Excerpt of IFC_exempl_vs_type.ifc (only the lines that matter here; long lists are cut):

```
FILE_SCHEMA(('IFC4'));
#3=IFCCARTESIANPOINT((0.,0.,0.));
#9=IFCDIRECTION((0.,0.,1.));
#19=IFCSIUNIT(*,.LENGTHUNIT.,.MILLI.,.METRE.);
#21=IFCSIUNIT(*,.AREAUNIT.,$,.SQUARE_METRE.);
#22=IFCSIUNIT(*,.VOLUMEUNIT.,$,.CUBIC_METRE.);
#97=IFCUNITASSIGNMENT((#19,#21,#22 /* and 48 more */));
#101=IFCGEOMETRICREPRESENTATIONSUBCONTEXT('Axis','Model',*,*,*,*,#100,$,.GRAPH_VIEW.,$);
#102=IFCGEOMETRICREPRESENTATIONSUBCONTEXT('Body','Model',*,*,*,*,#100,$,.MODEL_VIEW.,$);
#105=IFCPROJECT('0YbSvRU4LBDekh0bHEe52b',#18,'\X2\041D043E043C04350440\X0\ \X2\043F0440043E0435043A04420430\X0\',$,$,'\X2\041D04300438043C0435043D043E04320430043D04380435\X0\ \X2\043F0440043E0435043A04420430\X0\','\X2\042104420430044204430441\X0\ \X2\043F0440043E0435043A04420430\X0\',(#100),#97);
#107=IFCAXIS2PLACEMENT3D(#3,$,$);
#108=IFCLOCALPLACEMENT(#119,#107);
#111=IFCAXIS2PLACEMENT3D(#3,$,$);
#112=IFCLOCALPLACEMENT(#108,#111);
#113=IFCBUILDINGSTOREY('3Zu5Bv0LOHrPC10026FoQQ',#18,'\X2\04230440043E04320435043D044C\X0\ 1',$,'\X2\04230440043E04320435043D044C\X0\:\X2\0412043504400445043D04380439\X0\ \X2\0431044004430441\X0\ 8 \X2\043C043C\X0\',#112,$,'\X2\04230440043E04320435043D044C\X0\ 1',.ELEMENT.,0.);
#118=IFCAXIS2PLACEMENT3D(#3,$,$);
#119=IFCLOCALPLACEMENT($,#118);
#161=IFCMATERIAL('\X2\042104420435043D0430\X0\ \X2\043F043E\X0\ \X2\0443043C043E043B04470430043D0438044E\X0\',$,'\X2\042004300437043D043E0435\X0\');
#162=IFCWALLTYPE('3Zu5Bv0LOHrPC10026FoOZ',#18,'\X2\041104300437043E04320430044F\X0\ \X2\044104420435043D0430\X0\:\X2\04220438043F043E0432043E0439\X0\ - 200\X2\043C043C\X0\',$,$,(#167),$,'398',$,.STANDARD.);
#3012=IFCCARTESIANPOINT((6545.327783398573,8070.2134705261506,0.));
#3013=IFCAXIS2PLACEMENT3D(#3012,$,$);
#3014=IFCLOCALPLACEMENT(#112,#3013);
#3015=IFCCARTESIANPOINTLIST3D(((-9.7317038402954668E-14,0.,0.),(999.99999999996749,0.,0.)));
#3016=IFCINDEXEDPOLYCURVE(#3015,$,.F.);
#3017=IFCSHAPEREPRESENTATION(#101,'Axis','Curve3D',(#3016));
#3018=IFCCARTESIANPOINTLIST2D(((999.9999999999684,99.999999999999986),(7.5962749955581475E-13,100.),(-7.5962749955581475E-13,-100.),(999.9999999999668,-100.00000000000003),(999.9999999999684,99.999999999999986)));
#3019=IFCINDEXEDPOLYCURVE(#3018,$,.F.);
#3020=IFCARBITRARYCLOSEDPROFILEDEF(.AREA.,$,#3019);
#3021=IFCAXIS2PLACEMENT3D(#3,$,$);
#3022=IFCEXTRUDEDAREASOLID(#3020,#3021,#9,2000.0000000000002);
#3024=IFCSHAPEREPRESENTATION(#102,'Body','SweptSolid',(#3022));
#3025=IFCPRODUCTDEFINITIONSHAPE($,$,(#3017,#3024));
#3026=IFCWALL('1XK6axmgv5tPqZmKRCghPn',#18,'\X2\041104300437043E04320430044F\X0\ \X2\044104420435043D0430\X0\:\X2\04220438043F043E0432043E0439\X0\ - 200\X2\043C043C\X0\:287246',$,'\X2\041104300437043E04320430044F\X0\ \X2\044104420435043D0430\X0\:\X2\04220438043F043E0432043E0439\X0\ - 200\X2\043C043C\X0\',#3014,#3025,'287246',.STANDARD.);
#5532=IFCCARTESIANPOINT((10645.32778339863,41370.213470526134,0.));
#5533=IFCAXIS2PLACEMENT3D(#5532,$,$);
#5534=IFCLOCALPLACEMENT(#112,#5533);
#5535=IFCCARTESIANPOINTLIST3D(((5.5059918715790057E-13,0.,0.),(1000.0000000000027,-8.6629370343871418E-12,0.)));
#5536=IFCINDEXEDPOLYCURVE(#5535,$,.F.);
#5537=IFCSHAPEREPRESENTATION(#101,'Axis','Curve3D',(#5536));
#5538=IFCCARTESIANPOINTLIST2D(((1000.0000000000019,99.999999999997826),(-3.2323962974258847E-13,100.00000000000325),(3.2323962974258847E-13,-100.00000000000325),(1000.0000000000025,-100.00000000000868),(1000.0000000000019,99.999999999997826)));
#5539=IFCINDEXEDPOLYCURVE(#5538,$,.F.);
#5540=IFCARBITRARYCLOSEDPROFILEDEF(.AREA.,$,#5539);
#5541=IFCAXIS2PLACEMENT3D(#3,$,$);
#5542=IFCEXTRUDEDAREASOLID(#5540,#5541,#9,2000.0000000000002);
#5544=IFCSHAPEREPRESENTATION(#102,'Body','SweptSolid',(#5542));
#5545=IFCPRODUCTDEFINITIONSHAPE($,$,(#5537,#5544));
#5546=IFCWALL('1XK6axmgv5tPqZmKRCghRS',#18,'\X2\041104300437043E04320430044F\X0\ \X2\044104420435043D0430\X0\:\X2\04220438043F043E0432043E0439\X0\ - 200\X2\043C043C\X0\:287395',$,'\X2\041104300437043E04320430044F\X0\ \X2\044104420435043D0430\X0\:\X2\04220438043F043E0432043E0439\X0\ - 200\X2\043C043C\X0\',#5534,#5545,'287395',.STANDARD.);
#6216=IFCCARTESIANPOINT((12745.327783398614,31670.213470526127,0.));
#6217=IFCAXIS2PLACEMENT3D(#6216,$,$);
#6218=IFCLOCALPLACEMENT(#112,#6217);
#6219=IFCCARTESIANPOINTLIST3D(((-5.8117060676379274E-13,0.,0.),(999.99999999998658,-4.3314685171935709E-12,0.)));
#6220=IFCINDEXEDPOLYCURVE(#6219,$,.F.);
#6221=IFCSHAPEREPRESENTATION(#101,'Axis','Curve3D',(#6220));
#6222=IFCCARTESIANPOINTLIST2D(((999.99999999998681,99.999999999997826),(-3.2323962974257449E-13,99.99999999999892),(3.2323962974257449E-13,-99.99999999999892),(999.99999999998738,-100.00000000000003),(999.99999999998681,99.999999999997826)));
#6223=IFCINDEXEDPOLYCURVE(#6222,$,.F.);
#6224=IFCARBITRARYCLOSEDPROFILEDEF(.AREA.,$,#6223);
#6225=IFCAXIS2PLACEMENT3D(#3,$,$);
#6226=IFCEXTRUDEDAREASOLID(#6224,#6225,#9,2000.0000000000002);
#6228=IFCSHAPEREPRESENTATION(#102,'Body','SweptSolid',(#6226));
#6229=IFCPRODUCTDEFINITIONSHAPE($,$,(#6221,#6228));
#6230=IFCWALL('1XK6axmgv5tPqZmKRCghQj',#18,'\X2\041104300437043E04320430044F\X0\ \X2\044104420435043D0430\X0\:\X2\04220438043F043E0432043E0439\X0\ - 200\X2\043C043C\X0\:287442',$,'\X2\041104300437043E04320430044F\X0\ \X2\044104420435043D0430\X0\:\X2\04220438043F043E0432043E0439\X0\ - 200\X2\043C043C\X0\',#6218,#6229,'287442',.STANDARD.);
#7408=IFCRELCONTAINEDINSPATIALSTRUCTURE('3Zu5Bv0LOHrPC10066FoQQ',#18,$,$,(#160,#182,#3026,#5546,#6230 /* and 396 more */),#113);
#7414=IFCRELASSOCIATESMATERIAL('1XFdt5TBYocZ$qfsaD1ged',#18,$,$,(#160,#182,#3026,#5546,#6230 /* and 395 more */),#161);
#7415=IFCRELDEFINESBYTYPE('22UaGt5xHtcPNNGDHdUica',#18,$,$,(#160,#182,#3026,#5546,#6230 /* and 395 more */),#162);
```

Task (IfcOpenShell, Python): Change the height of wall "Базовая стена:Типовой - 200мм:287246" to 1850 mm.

```python
import ifcopenshell
import ifcopenshell.geom
import ifcopenshell.util.representation
import ifcopenshell.util.shape
import ifcopenshell.util.unit

model = ifcopenshell.open("IFC_exempl_vs_type.ifc")
unit_scale = ifcopenshell.util.unit.calculate_unit_scale(model)
settings = ifcopenshell.geom.settings()


def volume(element):
    """Net volume in cubic metres, openings subtracted."""
    shape = ifcopenshell.geom.create_shape(settings, element)
    return ifcopenshell.util.shape.get_volume(shape.geometry)


wall = model.by_guid("1XK6axmgv5tPqZmKRCghPn")
before = volume(wall)

body = ifcopenshell.util.representation.get_representation(wall, "Model", "Body")
solid = body.Items[0]
old_height = solid.Depth
solid.Depth = 1.85 / unit_scale
after = volume(wall)

print(f"height {old_height:g} -> {solid.Depth:g}, volume {before:.3f} -> {after:.3f} m3")

model.write("IFC_exempl_vs_type_edited.ifc")
```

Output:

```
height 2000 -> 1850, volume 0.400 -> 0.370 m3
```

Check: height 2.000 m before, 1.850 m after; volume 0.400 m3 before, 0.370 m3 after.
